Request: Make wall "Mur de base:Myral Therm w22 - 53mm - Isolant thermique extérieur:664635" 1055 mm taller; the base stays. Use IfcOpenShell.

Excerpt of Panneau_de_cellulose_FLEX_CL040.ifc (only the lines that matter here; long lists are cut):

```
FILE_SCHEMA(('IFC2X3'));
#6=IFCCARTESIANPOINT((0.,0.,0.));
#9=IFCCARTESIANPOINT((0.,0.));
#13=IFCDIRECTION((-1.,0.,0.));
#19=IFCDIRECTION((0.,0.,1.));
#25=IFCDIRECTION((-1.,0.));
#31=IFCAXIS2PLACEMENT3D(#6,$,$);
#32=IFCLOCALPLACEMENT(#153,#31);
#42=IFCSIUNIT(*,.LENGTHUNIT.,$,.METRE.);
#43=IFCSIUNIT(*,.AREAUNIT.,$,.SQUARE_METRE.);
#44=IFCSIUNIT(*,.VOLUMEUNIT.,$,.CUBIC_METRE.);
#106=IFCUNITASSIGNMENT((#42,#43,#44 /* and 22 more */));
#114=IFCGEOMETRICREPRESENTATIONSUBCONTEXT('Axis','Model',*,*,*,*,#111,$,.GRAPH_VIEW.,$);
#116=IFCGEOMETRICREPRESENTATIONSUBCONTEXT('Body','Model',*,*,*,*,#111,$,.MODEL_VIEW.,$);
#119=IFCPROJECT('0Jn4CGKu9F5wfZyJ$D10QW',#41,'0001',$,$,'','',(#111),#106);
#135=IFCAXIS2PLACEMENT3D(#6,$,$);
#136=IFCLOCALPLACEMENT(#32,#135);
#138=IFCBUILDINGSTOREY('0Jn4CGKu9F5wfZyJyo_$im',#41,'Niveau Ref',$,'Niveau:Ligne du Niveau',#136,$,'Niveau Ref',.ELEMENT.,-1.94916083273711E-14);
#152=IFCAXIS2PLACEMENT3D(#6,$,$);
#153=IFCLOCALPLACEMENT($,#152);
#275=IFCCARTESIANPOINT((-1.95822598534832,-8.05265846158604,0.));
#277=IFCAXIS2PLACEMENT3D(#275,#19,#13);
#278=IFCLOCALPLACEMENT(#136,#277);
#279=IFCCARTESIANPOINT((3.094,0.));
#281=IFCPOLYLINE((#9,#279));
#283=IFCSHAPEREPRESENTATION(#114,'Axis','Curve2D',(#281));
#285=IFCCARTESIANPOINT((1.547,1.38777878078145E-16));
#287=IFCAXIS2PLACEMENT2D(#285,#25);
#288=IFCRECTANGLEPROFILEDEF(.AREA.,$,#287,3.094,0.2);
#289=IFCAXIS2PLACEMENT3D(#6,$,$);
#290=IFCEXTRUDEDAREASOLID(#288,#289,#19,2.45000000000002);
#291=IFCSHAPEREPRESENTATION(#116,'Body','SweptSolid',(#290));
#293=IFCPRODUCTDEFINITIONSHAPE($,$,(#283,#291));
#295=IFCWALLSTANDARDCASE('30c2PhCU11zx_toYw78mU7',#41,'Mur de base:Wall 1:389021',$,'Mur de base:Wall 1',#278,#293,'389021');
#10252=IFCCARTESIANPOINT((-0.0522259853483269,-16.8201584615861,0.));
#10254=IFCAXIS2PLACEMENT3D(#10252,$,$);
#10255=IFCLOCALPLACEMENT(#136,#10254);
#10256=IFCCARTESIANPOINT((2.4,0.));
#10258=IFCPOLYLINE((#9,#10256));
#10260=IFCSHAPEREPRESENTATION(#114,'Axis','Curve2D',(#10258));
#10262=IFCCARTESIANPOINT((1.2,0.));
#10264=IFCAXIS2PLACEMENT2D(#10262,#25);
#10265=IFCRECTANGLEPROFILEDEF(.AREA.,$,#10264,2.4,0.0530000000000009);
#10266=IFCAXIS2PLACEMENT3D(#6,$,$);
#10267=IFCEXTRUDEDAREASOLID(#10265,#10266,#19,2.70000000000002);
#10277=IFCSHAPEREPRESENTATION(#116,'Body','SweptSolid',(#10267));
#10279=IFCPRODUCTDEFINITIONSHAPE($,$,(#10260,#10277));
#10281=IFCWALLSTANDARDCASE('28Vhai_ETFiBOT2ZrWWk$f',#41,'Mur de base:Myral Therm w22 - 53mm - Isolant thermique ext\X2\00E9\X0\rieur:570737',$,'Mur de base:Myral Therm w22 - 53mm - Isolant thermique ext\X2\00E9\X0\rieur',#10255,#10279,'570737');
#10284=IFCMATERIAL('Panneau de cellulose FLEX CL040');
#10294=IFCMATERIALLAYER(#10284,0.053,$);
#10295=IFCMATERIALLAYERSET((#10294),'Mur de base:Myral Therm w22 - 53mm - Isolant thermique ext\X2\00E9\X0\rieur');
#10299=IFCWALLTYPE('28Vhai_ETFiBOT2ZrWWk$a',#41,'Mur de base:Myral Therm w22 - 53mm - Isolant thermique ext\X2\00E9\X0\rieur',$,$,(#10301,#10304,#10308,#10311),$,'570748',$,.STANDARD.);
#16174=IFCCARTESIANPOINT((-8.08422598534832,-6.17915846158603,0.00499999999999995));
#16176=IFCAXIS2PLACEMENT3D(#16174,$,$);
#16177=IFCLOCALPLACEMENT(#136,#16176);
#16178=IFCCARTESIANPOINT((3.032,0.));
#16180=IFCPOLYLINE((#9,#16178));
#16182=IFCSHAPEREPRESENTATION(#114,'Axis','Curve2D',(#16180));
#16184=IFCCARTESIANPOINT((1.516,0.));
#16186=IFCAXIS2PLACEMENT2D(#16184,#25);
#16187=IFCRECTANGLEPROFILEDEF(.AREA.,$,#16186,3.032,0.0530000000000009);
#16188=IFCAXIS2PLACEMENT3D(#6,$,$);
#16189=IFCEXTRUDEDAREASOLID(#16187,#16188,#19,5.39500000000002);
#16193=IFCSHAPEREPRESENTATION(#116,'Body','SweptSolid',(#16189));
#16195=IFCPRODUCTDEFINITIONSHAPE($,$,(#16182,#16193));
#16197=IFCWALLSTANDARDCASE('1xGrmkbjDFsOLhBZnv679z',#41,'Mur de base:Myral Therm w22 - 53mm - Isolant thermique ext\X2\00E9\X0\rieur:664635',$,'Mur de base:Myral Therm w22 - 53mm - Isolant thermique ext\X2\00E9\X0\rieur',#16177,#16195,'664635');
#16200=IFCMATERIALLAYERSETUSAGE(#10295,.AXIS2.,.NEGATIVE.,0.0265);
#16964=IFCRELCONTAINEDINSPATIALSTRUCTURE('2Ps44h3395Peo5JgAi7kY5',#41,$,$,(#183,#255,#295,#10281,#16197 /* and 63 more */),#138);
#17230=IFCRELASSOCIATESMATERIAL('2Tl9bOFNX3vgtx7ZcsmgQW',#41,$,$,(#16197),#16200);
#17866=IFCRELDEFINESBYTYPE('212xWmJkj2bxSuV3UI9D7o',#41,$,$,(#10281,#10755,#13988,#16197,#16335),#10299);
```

```python
import ifcopenshell
import ifcopenshell.geom
import ifcopenshell.util.representation
import ifcopenshell.util.shape
import ifcopenshell.util.unit

model = ifcopenshell.open("Panneau_de_cellulose_FLEX_CL040.ifc")
unit_scale = ifcopenshell.util.unit.calculate_unit_scale(model)
settings = ifcopenshell.geom.settings()


def volume(element):
    """Net volume in cubic metres, openings subtracted."""
    shape = ifcopenshell.geom.create_shape(settings, element)
    return ifcopenshell.util.shape.get_volume(shape.geometry)


wall = model.by_guid("1xGrmkbjDFsOLhBZnv679z")
before = volume(wall)

body = ifcopenshell.util.representation.get_representation(wall, "Model", "Body")
solid = body.Items[0]
old_height = solid.Depth
solid.Depth += 1.055 / unit_scale
after = volume(wall)

print(f"height {old_height:g} -> {solid.Depth:g}, volume {before:.3f} -> {after:.3f} m3")

model.write("Panneau_de_cellulose_FLEX_CL040_v2.ifc")
```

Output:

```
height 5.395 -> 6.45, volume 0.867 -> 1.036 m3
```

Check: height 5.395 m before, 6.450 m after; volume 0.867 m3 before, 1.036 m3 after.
